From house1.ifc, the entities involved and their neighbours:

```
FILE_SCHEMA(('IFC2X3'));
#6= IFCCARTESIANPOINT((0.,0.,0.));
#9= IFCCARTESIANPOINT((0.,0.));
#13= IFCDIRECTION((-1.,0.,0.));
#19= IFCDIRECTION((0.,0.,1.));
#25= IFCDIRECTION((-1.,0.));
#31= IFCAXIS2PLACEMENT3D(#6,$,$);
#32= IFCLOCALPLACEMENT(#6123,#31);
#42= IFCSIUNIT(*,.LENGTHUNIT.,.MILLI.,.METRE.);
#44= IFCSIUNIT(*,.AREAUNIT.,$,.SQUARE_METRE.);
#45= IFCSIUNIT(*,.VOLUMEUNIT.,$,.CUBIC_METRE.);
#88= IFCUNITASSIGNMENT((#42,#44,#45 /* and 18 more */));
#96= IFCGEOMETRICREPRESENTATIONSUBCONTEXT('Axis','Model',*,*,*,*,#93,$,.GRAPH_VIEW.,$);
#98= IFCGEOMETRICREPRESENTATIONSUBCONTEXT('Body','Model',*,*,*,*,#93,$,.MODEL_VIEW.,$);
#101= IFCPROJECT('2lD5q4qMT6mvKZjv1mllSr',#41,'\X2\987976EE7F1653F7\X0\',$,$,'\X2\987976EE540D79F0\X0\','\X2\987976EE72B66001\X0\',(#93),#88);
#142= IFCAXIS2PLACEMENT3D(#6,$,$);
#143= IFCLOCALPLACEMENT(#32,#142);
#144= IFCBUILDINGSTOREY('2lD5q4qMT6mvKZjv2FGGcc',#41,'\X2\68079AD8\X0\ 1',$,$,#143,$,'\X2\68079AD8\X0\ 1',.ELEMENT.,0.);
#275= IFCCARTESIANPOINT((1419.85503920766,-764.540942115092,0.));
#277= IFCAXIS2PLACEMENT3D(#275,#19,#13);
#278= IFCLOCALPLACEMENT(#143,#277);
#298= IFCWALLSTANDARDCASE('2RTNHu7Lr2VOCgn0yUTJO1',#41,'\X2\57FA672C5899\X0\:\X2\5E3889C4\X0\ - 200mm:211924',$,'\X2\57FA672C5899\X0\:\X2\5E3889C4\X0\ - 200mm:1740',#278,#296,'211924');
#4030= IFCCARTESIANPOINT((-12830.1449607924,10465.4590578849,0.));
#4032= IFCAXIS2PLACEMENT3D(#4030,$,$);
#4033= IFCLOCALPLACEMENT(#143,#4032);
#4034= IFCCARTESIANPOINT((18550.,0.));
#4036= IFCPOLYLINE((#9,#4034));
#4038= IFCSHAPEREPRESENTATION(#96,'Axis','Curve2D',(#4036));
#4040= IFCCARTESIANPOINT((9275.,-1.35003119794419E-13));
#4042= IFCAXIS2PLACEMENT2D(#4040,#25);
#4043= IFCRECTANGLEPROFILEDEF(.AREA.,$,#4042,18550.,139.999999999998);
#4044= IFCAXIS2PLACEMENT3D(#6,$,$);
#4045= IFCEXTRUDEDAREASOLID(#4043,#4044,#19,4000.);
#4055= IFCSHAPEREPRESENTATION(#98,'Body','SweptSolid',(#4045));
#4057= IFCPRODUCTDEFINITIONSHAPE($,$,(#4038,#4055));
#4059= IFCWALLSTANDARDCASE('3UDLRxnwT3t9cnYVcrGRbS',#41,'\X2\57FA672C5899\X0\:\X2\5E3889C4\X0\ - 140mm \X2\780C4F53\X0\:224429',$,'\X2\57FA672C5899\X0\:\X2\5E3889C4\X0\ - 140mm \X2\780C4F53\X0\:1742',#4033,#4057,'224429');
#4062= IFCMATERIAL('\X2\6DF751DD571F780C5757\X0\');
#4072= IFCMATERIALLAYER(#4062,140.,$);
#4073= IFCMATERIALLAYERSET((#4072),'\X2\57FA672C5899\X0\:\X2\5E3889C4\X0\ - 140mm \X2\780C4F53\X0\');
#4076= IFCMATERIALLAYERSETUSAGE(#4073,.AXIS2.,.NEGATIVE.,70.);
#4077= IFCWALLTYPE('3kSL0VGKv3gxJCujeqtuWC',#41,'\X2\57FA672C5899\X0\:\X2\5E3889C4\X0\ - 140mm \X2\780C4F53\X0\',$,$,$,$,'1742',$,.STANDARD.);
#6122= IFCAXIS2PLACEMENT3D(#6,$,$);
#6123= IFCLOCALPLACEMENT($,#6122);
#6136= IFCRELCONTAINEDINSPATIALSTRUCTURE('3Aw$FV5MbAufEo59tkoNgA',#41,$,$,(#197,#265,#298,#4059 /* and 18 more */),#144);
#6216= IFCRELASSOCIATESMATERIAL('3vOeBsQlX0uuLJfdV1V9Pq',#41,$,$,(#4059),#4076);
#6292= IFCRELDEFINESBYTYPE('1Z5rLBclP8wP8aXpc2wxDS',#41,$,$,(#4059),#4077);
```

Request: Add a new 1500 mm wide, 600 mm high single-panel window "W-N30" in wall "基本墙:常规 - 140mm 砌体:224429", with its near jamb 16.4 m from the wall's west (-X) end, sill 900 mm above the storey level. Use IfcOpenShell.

```python
import numpy as np
import ifcopenshell
import ifcopenshell.api.feature
import ifcopenshell.api.geometry
import ifcopenshell.api.root
import ifcopenshell.api.spatial
import ifcopenshell.api.type
import ifcopenshell.geom
import ifcopenshell.util.element
import ifcopenshell.util.placement
import ifcopenshell.util.representation
import ifcopenshell.util.shape
import ifcopenshell.util.unit

model = ifcopenshell.open("house1.ifc")
unit_scale = ifcopenshell.util.unit.calculate_unit_scale(model)
settings = ifcopenshell.geom.settings()


def volume(element):
    """Net volume in cubic metres, openings subtracted."""
    shape = ifcopenshell.geom.create_shape(settings, element)
    return ifcopenshell.util.shape.get_volume(shape.geometry)


wall = model.by_id(4059)
storey = ifcopenshell.util.element.get_container(wall, ifc_class="IfcBuildingStorey")
context = ifcopenshell.util.representation.get_context(model, "Model", "Body", "MODEL_VIEW")
before = volume(wall)

width, height, from_end, sill = 1.5, 0.6, 16.4, 0.9  # metres

# The wall runs along its own X axis, and the end named is its -X end.
wall_shape = ifcopenshell.geom.create_shape(settings, wall)
x, y, z = ifcopenshell.util.shape.get_vertices(wall_shape.geometry).T
start = x.min() + from_end
face, thickness = float(y.min()), float(y.max() - y.min())
wall_matrix = ifcopenshell.util.placement.get_local_placement(wall.ObjectPlacement)
level = ifcopenshell.util.placement.get_local_placement(storey.ObjectPlacement)[2, 3]


def in_wall(x, y):
    """Placement at x, y metres in the wall's axes, at sill height."""
    matrix = wall_matrix.copy()
    matrix[:, 3] = wall_matrix @ np.array([x / unit_scale, y / unit_scale, 0.0, 1.0])
    matrix[2, 3] = level + sill / unit_scale
    return matrix


# Opening: a box that overshoots both wall faces by 50 mm.
opening = ifcopenshell.api.root.create_entity(model, ifc_class="IfcOpeningElement")
box = ifcopenshell.api.geometry.add_wall_representation(
    model, context=context, length=width, height=height, thickness=thickness + 0.1
)
ifcopenshell.api.geometry.assign_representation(model, product=opening, representation=box)
ifcopenshell.api.geometry.edit_object_placement(model, product=opening, matrix=in_wall(start, face - 0.05), is_si=False)
ifcopenshell.api.feature.add_feature(model, feature=opening, element=wall)

window = ifcopenshell.api.root.create_entity(model, ifc_class="IfcWindow", name="W-N30")
window.OverallWidth, window.OverallHeight = width / unit_scale, height / unit_scale
body = ifcopenshell.api.geometry.add_window_representation(
    model,
    context=context,
    overall_width=window.OverallWidth,
    overall_height=window.OverallHeight,
    partition_type="SINGLE_PANEL",
)
ifcopenshell.api.geometry.assign_representation(model, product=window, representation=body)
ifcopenshell.api.spatial.assign_container(model, products=[window], relating_structure=storey)
fills = ifcopenshell.api.feature.add_filling(model, opening=opening, element=window)
fills.OwnerHistory = window.OwnerHistory  # required in IFC2X3

# IFC2X3 keeps the operation on the window style.
style = ifcopenshell.api.root.create_entity(model, ifc_class="IfcWindowStyle", name="W-N30")
style.OperationType, style.ConstructionType = "SINGLE_PANEL", "NOTDEFINED"
style.ParameterTakesPrecedence = style.Sizeable = False
ifcopenshell.api.type.assign_type(model, related_objects=[window], relating_type=style)

# Centre the window in the wall's thickness.
ifcopenshell.api.geometry.edit_object_placement(model, product=window, matrix=in_wall(start, face), is_si=False)
window_shape = ifcopenshell.geom.create_shape(settings, window)
depth = ifcopenshell.util.shape.get_vertices(window_shape.geometry)[:, 1]
offset = face + thickness / 2 - (depth.min() + depth.max()) / 2
ifcopenshell.api.geometry.edit_object_placement(model, product=window, matrix=in_wall(start, offset), is_si=False)

after = volume(wall)

print(f"wall volume {before:.3f} -> {after:.3f} m3")

model.write("house1_updated.ifc")
```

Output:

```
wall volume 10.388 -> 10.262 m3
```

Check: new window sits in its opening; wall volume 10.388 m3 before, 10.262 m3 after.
